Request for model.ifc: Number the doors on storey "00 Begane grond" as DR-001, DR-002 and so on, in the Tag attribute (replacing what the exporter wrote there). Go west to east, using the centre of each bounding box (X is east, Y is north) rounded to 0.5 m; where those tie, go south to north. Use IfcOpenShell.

First a look at what the model holds.

```python
import ifcopenshell
import ifcopenshell.util.element
import ifcopenshell.util.placement

model = ifcopenshell.open("model.ifc")
print(model.schema)
storey = next(s for s in model.by_type("IfcBuildingStorey") if s.Name == "00 Begane grond")
doors = [e for e in ifcopenshell.util.element.get_decomposition(storey) if e.is_a("IfcDoor")]
for e in sorted(doors, key=lambda e: e.id()):
    origin = ifcopenshell.util.placement.get_local_placement(e.ObjectPlacement)[:3, 3]
    print(e.id(), e.Tag, e.Name, origin.round(2) + 0.0, sep=" | ")
```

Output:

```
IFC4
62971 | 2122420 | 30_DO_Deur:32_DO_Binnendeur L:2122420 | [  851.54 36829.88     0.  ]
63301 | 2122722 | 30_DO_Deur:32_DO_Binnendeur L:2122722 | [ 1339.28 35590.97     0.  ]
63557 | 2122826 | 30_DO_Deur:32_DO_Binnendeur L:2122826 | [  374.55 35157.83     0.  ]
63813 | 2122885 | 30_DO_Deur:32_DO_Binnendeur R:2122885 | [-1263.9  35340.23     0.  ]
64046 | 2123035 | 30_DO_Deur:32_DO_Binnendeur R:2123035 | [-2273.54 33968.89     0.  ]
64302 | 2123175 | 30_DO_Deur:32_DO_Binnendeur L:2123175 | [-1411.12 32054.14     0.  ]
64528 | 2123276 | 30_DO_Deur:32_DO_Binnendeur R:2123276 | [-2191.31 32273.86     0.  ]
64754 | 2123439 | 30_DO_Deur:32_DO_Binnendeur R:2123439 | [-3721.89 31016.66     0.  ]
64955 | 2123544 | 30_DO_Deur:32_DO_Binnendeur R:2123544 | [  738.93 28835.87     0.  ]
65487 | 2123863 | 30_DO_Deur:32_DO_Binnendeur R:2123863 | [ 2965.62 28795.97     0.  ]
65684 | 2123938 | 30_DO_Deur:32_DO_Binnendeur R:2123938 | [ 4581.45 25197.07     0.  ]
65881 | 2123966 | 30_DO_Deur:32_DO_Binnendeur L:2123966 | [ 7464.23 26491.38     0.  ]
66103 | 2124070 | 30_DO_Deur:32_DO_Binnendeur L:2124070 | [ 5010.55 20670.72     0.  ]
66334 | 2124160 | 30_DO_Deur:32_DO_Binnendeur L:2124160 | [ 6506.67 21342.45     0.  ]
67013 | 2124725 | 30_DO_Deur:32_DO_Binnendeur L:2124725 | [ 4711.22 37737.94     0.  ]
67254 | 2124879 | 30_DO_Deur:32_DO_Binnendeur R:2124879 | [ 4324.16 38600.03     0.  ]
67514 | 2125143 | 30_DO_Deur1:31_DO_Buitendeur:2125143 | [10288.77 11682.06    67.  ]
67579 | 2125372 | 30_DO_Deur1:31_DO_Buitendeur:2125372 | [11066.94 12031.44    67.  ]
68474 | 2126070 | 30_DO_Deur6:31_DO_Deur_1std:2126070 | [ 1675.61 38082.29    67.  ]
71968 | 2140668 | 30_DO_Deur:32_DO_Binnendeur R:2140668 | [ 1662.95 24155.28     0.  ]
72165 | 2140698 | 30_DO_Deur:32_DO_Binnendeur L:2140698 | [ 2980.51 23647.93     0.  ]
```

```python
import ifcopenshell
import ifcopenshell.geom
import ifcopenshell.util.element
import ifcopenshell.util.shape

model = ifcopenshell.open("model.ifc")
settings = ifcopenshell.geom.settings()
settings.set("use-world-coords", True)


def centre(element):
    shape = ifcopenshell.geom.create_shape(settings, element)
    return ifcopenshell.util.shape.get_bbox_centroid(shape.geometry)


storey = next(s for s in model.by_type("IfcBuildingStorey") if s.Name == "00 Begane grond")
doors = [e for e in ifcopenshell.util.element.get_decomposition(storey) if e.is_a("IfcDoor")]

# Insertion points can sit at a corner or the storey origin, so sort by the geometry (in metres).
centres = {e: centre(e) for e in doors}
doors.sort(key=lambda e: (round(centres[e][0] / 0.5), centres[e][1]))

for i, e in enumerate(doors, start=1):
    number = f"DR-0{i:02d}"
    e.Tag = number
    print(e.id(), number)

model.write("model_updated.ifc")
```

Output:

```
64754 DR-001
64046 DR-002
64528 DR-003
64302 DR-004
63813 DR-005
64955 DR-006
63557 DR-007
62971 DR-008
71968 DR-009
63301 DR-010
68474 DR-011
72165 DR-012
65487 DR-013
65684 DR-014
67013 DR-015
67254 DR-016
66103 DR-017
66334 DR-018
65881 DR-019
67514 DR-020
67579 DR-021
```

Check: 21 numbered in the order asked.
